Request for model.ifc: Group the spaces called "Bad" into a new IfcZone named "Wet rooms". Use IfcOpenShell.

First a look at what the model holds.

```python
import ifcopenshell

model = ifcopenshell.open("model.ifc")
print(model.schema)
seen = {}
for space in model.by_type("IfcSpace"):
    seen[space.LongName] = seen.get(space.LongName, 0) + 1
for name, count in sorted(seen.items(), key=str):
    print(count, "x", name)
print("zones:", [z.Name for z in model.by_type("IfcZone")][:20])
```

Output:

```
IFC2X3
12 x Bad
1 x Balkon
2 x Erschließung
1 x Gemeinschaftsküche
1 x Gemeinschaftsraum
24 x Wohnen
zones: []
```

```python
import ifcopenshell
import ifcopenshell.api.group
import ifcopenshell.api.root

model = ifcopenshell.open("model.ifc")

names = {"Bad"}
spaces = [s for s in model.by_type("IfcSpace") if s.LongName in names]

zone = ifcopenshell.api.root.create_entity(model, ifc_class="IfcZone", name="Wet rooms")
ifcopenshell.api.group.assign_group(model, products=spaces, group=zone)
print(len(spaces), "spaces in", zone.Name)

model.write("model_rev.ifc")
```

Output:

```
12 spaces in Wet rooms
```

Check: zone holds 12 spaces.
